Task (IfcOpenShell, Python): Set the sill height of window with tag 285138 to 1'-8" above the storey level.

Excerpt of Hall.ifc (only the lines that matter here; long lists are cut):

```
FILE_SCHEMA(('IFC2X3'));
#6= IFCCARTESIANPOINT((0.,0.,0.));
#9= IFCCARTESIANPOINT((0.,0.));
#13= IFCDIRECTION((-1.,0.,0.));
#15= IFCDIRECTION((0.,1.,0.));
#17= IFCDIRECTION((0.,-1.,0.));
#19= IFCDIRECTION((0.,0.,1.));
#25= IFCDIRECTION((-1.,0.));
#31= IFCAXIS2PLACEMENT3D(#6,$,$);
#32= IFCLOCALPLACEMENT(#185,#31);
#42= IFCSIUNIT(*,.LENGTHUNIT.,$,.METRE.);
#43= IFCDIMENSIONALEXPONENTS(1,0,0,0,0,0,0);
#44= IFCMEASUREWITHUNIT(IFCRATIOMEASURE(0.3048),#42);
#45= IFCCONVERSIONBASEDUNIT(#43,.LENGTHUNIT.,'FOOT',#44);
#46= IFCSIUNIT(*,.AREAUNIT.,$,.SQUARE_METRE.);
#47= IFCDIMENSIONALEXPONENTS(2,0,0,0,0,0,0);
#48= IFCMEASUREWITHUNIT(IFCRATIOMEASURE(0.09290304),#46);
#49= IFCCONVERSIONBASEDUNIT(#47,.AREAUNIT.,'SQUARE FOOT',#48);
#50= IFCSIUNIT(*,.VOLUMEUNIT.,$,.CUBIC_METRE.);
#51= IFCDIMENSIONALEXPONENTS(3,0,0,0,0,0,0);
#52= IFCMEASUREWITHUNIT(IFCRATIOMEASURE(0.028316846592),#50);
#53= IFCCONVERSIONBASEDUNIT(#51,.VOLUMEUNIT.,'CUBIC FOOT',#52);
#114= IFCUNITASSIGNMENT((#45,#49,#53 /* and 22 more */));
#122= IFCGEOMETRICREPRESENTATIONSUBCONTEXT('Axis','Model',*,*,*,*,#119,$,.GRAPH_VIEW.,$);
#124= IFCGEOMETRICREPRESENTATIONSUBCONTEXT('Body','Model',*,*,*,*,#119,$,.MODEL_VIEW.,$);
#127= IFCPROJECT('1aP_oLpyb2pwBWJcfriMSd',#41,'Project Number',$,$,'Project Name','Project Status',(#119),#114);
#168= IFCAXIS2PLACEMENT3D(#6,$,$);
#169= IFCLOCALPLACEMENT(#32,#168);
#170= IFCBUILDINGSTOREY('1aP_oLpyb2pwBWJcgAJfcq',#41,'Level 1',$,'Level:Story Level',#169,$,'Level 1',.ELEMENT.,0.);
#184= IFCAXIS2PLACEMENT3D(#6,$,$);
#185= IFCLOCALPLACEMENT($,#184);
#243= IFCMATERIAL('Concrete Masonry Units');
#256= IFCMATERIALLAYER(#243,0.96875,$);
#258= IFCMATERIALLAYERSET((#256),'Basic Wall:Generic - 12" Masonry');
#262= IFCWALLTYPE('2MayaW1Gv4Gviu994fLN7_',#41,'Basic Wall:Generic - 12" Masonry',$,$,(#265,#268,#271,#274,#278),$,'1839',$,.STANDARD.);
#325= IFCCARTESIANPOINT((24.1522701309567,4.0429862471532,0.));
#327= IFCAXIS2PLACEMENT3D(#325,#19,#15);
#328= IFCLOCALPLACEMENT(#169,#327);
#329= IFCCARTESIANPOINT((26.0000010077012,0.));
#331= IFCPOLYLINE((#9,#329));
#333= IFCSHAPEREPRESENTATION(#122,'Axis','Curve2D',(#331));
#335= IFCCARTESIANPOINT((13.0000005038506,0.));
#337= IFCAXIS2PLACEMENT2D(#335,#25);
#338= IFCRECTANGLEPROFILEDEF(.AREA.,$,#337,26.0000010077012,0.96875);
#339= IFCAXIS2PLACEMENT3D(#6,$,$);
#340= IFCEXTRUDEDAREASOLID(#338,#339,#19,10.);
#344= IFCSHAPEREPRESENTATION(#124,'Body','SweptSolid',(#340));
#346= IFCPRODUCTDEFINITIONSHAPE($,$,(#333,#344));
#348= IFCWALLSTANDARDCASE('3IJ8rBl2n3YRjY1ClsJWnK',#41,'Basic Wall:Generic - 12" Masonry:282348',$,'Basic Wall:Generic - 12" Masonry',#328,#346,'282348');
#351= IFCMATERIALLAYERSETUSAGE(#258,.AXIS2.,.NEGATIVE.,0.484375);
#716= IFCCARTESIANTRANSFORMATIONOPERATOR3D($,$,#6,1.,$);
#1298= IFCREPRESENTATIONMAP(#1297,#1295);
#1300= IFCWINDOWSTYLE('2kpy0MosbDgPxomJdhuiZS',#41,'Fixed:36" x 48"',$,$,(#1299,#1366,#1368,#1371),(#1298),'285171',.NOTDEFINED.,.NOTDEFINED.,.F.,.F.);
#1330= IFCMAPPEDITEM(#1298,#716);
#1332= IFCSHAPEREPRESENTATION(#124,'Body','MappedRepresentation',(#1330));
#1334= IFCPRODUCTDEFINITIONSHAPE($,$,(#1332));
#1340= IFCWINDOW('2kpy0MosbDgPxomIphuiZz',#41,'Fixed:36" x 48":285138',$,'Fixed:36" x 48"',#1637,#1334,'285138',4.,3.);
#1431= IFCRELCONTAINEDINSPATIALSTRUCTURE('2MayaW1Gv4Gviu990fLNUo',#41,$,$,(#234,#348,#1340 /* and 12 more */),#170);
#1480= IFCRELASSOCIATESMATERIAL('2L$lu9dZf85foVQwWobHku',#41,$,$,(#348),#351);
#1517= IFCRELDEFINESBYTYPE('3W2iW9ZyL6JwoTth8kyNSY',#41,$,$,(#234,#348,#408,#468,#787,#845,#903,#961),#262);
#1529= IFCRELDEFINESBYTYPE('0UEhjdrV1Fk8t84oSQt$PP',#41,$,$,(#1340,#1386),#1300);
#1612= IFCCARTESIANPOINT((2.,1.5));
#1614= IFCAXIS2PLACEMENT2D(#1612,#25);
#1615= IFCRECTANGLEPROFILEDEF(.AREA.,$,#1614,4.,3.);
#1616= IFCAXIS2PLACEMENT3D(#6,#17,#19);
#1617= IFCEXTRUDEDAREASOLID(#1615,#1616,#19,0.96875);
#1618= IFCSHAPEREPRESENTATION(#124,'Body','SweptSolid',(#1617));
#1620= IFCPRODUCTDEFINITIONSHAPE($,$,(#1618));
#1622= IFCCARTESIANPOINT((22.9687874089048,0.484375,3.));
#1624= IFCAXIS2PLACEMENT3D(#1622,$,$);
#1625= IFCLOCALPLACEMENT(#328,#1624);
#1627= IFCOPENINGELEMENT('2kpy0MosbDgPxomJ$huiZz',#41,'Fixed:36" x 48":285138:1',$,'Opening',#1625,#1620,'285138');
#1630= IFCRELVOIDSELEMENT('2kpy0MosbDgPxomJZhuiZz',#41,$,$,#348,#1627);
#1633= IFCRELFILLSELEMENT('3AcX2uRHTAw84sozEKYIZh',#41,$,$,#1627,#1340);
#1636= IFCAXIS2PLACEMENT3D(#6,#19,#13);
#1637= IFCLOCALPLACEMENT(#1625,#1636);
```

```python
import numpy as np
import ifcopenshell
import ifcopenshell.api.geometry
import ifcopenshell.geom
import ifcopenshell.util.element
import ifcopenshell.util.placement
import ifcopenshell.util.shape
import ifcopenshell.util.unit

model = ifcopenshell.open("Hall.ifc")
unit_scale = ifcopenshell.util.unit.calculate_unit_scale(model)

window = model.by_guid("2kpy0MosbDgPxomIphuiZz")
opening = window.FillsVoids[0].RelatingOpeningElement
storey = ifcopenshell.util.element.get_container(window, ifc_class="IfcBuildingStorey")
level = ifcopenshell.util.placement.get_local_placement(storey.ObjectPlacement)[2, 3]

# The opening's origin need not be at the sill, so measure its lowest point.
shape = ifcopenshell.geom.create_shape(ifcopenshell.geom.settings(), opening)
bottom = ifcopenshell.util.shape.get_shape_bottom_elevation(shape, shape.geometry) / unit_scale
dz = level + 20 * 0.0254 / unit_scale - bottom

shift = np.array([0.0, 0.0, dz])
# The window is placed relative to its opening, so it follows when the opening moves.
matrix = ifcopenshell.util.placement.get_local_placement(opening.ObjectPlacement)
matrix[:3, 3] += shift
ifcopenshell.api.geometry.edit_object_placement(
    model, product=opening, matrix=matrix, is_si=False, should_transform_children=True
)

print(f"moved by {dz * unit_scale:+.3f} m")

model.write("Hall_updated.ifc")
```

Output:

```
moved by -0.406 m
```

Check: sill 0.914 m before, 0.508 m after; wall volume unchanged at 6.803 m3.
